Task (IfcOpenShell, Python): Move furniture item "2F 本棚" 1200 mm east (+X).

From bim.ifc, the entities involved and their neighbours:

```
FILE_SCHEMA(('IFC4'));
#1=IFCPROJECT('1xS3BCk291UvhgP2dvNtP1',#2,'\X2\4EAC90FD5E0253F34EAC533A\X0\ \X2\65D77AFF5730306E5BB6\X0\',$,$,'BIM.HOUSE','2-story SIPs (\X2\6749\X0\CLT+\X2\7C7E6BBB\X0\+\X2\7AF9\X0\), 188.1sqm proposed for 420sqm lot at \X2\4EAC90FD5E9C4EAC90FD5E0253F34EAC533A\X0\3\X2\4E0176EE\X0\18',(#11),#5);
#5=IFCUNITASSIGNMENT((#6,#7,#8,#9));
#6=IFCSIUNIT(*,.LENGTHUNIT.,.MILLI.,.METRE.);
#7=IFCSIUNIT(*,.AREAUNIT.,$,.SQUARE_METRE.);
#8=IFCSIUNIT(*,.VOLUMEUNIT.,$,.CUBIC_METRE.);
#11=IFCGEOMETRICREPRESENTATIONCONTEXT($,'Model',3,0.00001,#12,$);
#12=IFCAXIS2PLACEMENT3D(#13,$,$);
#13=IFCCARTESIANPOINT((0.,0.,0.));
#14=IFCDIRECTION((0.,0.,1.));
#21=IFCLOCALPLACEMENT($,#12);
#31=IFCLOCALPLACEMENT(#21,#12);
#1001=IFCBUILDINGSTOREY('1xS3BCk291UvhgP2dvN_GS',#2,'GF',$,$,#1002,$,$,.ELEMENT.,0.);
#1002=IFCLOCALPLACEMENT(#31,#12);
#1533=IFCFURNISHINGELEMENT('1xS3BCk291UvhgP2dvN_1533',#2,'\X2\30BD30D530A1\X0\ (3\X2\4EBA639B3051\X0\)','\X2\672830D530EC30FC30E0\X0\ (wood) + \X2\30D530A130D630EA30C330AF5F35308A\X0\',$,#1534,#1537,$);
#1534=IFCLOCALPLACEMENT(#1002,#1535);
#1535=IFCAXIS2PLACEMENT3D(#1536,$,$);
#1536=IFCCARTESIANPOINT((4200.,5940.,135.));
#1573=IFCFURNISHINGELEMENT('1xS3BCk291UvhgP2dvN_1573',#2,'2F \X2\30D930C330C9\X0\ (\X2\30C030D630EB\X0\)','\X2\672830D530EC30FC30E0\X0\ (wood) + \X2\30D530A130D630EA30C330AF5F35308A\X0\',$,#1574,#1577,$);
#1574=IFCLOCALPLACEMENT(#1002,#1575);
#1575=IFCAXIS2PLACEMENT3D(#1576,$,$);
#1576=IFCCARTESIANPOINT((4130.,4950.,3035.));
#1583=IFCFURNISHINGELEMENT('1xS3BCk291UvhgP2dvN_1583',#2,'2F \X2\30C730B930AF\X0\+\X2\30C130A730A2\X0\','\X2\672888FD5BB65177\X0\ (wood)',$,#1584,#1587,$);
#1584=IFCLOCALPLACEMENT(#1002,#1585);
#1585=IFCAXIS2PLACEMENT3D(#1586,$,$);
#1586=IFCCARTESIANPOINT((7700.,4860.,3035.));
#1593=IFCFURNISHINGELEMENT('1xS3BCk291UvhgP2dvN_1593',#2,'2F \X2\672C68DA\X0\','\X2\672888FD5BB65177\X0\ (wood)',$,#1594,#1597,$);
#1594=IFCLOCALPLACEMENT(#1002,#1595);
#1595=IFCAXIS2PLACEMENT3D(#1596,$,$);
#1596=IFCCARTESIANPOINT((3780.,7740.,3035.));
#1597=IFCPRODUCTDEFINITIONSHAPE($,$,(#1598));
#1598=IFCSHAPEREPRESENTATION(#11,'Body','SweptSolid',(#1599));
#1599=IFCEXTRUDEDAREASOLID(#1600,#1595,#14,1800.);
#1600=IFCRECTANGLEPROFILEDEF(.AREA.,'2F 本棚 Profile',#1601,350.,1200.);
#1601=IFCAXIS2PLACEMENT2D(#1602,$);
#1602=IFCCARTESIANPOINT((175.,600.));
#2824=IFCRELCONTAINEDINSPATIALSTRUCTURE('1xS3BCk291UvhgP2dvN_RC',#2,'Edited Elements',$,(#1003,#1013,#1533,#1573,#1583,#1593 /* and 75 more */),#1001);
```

```python
import ifcopenshell
import ifcopenshell.api.geometry
import ifcopenshell.util.placement
import ifcopenshell.util.unit

model = ifcopenshell.open("bim.ifc")
unit_scale = ifcopenshell.util.unit.calculate_unit_scale(model)

item = model.by_guid("1xS3BCk291UvhgP2dvN_1593")
matrix = ifcopenshell.util.placement.get_local_placement(item.ObjectPlacement)
matrix[0, 3] += 1.2 / unit_scale
ifcopenshell.api.geometry.edit_object_placement(model, product=item, matrix=matrix, is_si=False)

print(ifcopenshell.util.placement.get_local_placement(item.ObjectPlacement).round(3) + 0.0)

model.write("bim_edited.ifc")
```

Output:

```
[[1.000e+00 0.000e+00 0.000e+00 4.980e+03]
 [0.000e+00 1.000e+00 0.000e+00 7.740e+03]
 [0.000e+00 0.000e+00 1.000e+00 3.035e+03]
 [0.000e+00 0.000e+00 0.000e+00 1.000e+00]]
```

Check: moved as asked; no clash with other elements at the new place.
